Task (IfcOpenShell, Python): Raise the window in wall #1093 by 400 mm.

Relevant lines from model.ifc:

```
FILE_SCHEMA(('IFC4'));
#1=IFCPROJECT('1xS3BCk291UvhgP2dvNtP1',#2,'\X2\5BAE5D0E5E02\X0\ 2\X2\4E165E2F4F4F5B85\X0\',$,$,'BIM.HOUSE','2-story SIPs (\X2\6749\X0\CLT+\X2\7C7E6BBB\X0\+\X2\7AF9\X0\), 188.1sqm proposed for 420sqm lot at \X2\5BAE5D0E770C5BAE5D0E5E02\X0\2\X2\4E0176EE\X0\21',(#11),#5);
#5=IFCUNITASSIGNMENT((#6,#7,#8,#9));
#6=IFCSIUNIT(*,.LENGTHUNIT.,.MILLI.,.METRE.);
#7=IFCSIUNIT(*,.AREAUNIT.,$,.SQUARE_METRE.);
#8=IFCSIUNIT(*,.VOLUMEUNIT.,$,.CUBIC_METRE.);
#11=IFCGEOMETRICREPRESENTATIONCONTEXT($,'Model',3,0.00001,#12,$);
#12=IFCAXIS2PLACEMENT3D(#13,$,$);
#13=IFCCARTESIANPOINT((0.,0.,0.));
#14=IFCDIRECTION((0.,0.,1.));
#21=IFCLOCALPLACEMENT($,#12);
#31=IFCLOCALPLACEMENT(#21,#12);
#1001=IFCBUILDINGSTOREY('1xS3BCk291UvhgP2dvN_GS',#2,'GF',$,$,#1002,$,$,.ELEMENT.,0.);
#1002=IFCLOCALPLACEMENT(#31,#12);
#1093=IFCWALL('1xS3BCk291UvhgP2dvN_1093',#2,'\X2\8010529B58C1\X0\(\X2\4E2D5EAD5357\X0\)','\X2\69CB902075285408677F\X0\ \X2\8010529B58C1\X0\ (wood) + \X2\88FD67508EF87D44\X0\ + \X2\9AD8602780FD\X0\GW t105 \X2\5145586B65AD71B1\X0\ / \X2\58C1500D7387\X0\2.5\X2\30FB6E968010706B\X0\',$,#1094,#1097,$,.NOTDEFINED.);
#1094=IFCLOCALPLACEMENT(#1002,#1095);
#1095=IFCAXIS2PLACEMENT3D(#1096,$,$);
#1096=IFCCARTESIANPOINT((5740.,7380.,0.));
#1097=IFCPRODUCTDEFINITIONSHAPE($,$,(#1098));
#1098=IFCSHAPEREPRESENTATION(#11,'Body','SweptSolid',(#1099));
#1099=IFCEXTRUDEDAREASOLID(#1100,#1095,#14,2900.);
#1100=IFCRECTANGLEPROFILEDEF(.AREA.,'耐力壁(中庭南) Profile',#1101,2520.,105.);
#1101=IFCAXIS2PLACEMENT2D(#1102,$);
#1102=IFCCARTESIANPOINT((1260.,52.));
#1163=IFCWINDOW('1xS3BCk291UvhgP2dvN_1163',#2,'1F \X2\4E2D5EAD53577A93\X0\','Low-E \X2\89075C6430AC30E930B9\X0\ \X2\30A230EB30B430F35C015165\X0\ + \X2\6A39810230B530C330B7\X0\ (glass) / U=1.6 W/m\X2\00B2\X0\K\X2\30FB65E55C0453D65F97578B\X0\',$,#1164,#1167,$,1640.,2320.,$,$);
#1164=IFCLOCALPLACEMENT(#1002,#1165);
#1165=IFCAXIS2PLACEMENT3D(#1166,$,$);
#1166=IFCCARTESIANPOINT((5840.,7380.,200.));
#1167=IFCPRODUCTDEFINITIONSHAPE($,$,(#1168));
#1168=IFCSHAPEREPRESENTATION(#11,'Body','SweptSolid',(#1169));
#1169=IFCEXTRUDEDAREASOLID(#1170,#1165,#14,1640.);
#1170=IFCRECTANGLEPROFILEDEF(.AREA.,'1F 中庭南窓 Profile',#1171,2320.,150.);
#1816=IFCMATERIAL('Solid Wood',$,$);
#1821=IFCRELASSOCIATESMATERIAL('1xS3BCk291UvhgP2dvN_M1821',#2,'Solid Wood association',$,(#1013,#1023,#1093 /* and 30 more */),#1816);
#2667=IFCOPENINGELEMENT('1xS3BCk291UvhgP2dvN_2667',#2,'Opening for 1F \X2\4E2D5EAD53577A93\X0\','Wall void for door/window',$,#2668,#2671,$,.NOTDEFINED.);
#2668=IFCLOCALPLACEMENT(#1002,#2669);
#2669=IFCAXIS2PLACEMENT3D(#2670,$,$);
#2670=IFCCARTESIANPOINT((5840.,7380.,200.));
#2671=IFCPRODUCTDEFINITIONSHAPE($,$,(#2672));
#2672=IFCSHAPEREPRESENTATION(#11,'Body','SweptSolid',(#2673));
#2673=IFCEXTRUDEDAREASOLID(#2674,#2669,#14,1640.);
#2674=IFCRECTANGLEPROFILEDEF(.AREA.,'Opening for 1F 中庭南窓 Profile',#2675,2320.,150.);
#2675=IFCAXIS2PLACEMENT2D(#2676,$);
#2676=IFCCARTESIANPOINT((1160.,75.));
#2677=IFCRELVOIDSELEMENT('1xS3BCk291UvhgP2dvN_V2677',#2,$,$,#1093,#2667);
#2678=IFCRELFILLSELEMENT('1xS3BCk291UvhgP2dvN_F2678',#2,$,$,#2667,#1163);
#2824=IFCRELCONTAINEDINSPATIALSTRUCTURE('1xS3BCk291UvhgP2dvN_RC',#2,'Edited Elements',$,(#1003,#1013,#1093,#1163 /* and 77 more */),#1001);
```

```python
import numpy as np
import ifcopenshell
import ifcopenshell.api.geometry
import ifcopenshell.util.placement
import ifcopenshell.util.unit

model = ifcopenshell.open("model.ifc")
unit_scale = ifcopenshell.util.unit.calculate_unit_scale(model)

window = model.by_guid("1xS3BCk291UvhgP2dvN_1163")
opening = window.FillsVoids[0].RelatingOpeningElement
dz = 0.4 / unit_scale

shift = np.array([0.0, 0.0, dz])
# The window is not placed relative to its opening, so move both.
for product in (opening, window):
    matrix = ifcopenshell.util.placement.get_local_placement(product.ObjectPlacement)
    matrix[:3, 3] += shift
    ifcopenshell.api.geometry.edit_object_placement(model, product=product, matrix=matrix, is_si=False)

print(f"moved by {dz * unit_scale:+.3f} m")

model.write("model_v2.ifc")
```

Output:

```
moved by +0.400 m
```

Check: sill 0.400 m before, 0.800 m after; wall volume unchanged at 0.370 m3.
